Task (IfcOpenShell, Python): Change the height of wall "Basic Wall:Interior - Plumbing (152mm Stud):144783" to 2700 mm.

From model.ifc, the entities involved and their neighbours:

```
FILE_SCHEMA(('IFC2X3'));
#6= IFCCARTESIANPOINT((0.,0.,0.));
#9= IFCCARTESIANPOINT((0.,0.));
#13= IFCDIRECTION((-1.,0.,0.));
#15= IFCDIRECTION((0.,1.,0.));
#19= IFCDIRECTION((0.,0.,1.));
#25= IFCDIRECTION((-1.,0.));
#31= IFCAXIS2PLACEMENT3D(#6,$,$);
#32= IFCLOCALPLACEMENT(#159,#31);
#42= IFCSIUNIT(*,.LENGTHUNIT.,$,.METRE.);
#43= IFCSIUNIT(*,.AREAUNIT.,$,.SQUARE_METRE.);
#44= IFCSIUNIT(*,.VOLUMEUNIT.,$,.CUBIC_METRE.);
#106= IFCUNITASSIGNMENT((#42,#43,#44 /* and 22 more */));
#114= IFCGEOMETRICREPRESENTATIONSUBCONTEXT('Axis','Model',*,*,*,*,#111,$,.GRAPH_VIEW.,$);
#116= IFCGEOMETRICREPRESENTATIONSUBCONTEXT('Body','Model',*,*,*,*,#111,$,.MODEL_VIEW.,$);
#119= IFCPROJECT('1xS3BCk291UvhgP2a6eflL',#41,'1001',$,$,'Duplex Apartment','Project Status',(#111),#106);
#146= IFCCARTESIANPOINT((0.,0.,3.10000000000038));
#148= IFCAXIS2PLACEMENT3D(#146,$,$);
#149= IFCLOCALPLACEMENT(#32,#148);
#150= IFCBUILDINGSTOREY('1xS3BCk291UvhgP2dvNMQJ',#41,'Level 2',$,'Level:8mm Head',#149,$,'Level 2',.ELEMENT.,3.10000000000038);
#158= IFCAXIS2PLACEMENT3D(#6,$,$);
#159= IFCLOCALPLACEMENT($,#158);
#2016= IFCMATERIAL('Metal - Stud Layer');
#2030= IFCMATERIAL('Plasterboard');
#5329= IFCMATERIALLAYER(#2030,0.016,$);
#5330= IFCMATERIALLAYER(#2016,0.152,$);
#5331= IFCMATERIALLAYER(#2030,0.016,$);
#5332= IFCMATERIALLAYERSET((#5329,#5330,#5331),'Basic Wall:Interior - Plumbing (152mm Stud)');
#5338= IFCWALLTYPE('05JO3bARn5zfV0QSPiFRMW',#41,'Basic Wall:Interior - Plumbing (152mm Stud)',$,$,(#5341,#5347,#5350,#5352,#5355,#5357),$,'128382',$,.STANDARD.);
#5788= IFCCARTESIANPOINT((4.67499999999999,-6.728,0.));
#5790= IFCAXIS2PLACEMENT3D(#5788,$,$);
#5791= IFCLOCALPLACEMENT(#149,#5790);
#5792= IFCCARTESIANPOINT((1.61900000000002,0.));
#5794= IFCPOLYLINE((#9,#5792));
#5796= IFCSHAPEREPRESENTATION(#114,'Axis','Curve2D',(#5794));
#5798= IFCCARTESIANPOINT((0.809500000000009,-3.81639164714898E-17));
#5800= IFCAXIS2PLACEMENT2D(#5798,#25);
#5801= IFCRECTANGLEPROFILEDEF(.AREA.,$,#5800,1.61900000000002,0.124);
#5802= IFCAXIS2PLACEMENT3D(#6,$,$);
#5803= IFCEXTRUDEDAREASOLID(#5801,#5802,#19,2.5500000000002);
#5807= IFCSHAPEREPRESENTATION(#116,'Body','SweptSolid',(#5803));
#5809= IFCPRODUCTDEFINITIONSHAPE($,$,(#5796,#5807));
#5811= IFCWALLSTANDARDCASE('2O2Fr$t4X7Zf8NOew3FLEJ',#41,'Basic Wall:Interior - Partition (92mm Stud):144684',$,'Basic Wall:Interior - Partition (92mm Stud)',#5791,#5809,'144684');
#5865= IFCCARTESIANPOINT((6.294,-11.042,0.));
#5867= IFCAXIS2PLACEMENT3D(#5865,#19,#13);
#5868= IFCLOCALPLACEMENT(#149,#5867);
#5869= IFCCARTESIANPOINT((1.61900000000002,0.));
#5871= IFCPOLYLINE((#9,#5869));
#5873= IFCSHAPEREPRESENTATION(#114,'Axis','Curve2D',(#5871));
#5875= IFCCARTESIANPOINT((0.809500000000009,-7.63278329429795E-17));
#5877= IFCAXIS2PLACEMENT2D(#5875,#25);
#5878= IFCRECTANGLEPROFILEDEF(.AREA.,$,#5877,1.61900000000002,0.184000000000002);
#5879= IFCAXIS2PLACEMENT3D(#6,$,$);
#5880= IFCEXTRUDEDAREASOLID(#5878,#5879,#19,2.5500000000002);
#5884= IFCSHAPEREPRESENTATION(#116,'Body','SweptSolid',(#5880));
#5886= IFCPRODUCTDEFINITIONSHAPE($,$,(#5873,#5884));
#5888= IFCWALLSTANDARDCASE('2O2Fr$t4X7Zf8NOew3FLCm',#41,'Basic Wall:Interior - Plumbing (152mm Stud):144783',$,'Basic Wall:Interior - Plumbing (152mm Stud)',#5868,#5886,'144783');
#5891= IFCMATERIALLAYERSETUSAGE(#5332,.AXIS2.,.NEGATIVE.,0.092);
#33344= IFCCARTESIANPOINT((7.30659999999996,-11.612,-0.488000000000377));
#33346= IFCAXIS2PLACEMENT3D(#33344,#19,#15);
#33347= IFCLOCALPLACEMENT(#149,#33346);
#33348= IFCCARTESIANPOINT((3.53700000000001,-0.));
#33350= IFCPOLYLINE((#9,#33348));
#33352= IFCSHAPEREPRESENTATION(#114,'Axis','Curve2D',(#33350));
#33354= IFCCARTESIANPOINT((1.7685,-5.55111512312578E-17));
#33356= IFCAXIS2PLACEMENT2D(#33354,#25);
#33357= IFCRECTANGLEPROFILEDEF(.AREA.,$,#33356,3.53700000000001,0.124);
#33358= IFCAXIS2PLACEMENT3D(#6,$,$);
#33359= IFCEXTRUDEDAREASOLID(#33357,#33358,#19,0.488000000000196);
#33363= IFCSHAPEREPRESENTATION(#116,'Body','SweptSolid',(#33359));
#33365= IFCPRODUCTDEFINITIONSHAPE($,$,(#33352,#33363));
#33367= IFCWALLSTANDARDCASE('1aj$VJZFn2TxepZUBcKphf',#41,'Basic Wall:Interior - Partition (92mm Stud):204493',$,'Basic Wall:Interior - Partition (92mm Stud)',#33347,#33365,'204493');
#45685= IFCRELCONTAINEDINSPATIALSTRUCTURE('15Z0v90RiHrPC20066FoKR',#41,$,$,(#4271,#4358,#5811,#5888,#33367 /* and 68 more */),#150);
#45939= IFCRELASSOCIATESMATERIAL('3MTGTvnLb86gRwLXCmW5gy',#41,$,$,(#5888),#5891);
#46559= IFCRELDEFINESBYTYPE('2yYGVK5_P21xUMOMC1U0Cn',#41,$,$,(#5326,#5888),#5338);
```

```python
import ifcopenshell
import ifcopenshell.geom
import ifcopenshell.util.representation
import ifcopenshell.util.shape
import ifcopenshell.util.unit

model = ifcopenshell.open("model.ifc")
unit_scale = ifcopenshell.util.unit.calculate_unit_scale(model)
settings = ifcopenshell.geom.settings()


def volume(element):
    """Net volume in cubic metres, openings subtracted."""
    shape = ifcopenshell.geom.create_shape(settings, element)
    return ifcopenshell.util.shape.get_volume(shape.geometry)


wall = model.by_guid("2O2Fr$t4X7Zf8NOew3FLCm")
before = volume(wall)

body = ifcopenshell.util.representation.get_representation(wall, "Model", "Body")
solid = body.Items[0]
old_height = solid.Depth
solid.Depth = 2.7 / unit_scale
after = volume(wall)

print(f"height {old_height:g} -> {solid.Depth:g}, volume {before:.3f} -> {after:.3f} m3")

model.write("model_updated.ifc")
```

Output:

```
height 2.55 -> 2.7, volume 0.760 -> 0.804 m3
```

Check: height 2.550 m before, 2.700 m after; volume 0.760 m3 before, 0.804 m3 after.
